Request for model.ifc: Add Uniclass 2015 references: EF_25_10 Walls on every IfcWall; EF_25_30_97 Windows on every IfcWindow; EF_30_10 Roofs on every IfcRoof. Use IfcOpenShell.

First a look at what the model holds.

```python
import ifcopenshell

model = ifcopenshell.open("model.ifc")
print(model.schema)
print("classifications:", [c.Name for c in model.by_type("IfcClassification")])
for ifc_class in ("IfcDoor", "IfcRoof", "IfcStair", "IfcWall", "IfcWindow"):
    print(ifc_class, len(model.by_type(ifc_class)))
```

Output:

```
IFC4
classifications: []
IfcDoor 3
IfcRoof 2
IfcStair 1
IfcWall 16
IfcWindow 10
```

```python
import ifcopenshell
import ifcopenshell.api.classification

model = ifcopenshell.open("model.ifc")

system = ifcopenshell.api.classification.add_classification(model, classification="Uniclass 2015")

codes = {
    "IfcWall": ("EF_25_10", "Walls"),
    "IfcWindow": ("EF_25_30_97", "Windows"),
    "IfcRoof": ("EF_30_10", "Roofs"),
}
for ifc_class, (code, name) in codes.items():
    products = model.by_type(ifc_class)
    ifcopenshell.api.classification.add_reference(
        model, products=products, classification=system, identification=code, name=name
    )
    print(code, len(products))

model.write("model_updated.ifc")
```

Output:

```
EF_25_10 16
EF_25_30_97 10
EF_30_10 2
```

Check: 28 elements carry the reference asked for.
